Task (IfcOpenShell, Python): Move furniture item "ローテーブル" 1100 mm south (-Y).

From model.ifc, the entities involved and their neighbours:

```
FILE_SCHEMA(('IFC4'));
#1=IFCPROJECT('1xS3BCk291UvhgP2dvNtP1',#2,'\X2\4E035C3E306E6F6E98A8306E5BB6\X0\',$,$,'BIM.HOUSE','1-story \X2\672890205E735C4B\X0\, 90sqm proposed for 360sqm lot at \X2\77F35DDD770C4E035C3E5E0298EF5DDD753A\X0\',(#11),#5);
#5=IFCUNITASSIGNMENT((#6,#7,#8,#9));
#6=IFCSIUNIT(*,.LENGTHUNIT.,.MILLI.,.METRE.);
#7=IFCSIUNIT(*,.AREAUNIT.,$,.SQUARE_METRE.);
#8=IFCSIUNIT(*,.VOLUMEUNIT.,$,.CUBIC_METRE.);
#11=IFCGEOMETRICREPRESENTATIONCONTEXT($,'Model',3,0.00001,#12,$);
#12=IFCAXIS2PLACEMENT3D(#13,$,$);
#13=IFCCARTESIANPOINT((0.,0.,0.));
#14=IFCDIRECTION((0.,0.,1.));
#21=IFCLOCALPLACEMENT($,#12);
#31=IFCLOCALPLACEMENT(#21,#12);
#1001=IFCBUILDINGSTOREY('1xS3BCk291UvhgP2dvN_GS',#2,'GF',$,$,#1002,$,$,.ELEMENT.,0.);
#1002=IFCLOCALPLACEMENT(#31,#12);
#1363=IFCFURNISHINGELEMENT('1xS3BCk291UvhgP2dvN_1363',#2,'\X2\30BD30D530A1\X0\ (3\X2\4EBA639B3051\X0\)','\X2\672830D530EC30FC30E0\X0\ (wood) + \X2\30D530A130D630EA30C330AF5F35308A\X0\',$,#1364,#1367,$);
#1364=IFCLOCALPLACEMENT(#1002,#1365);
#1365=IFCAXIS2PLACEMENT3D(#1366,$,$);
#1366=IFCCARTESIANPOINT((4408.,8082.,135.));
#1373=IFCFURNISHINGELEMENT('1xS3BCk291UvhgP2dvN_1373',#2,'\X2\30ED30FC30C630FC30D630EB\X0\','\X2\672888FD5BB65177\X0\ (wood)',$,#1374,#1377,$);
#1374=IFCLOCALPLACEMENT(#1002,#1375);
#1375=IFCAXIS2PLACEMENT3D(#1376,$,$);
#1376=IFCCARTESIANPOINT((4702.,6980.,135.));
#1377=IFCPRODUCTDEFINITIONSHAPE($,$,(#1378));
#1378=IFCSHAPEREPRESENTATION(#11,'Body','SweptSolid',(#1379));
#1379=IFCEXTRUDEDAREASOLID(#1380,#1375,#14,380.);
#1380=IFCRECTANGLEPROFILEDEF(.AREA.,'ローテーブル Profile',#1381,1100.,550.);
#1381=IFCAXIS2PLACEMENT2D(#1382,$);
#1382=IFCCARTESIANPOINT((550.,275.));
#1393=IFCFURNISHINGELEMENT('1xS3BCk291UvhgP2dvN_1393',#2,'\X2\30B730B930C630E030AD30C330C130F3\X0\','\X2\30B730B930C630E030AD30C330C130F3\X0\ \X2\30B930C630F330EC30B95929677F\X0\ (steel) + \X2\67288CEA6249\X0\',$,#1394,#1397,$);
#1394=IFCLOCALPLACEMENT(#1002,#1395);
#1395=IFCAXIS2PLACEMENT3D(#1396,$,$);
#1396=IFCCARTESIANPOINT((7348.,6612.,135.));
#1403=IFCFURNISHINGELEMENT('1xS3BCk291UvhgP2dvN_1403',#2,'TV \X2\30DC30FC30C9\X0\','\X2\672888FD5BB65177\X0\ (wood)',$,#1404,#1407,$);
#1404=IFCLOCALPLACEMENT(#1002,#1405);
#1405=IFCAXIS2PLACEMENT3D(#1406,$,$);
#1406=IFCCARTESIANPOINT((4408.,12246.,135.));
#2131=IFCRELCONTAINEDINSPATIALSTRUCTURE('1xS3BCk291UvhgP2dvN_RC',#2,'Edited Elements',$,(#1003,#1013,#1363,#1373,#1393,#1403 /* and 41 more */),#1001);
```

```python
import ifcopenshell
import ifcopenshell.api.geometry
import ifcopenshell.util.placement

model = ifcopenshell.open("model.ifc")

item = model.by_id(1373)
matrix = ifcopenshell.util.placement.get_local_placement(item.ObjectPlacement)
matrix[1, 3] -= 1100.0
ifcopenshell.api.geometry.edit_object_placement(model, product=item, matrix=matrix, is_si=False)

print(ifcopenshell.util.placement.get_local_placement(item.ObjectPlacement).round(3) + 0.0)

model.write("model-out.ifc")
```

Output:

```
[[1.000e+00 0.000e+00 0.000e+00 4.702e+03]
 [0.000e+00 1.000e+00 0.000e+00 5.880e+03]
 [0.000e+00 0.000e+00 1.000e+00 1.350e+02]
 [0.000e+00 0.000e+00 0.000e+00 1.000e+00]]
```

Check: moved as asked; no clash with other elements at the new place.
